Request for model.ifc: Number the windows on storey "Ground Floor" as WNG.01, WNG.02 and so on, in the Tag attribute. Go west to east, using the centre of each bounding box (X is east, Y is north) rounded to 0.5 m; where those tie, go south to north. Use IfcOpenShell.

First a look at what the model holds.

```python
import ifcopenshell
import ifcopenshell.util.element
import ifcopenshell.util.placement

model = ifcopenshell.open("model.ifc")
print(model.schema)
storey = next(s for s in model.by_type("IfcBuildingStorey") if s.Name == "Ground Floor")
windows = [e for e in ifcopenshell.util.element.get_decomposition(storey) if e.is_a("IfcWindow")]
for e in sorted(windows, key=lambda e: e.id()):
    origin = ifcopenshell.util.placement.get_local_placement(e.ObjectPlacement)[:3, 3]
    print(e.id(), e.Tag, e.Name, origin.round(2) + 0.0, sep=" | ")
```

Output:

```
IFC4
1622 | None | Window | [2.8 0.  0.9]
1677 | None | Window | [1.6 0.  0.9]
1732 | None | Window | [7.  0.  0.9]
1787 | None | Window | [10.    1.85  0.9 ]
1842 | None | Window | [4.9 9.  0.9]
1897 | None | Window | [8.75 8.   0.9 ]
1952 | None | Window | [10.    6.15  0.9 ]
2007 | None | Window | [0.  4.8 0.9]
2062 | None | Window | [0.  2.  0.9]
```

```python
import ifcopenshell
import ifcopenshell.geom
import ifcopenshell.util.element
import ifcopenshell.util.shape

model = ifcopenshell.open("model.ifc")
settings = ifcopenshell.geom.settings()
settings.set("use-world-coords", True)


def centre(element):
    shape = ifcopenshell.geom.create_shape(settings, element)
    return ifcopenshell.util.shape.get_bbox_centroid(shape.geometry)


storey = next(s for s in model.by_type("IfcBuildingStorey") if s.Name == "Ground Floor")
windows = [e for e in ifcopenshell.util.element.get_decomposition(storey) if e.is_a("IfcWindow")]

# Insertion points can sit at a corner or the storey origin, so sort by the geometry (in metres).
centres = {e: centre(e) for e in windows}
windows.sort(key=lambda e: (round(centres[e][0] / 0.5), centres[e][1]))

for i, e in enumerate(windows, start=1):
    number = f"WNG.{i:02d}"
    e.Tag = number
    print(e.id(), number)

model.write("model_rev.ifc")
```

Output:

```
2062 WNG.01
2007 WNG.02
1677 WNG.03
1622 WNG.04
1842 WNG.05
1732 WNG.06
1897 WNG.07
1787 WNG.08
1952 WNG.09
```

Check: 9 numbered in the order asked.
